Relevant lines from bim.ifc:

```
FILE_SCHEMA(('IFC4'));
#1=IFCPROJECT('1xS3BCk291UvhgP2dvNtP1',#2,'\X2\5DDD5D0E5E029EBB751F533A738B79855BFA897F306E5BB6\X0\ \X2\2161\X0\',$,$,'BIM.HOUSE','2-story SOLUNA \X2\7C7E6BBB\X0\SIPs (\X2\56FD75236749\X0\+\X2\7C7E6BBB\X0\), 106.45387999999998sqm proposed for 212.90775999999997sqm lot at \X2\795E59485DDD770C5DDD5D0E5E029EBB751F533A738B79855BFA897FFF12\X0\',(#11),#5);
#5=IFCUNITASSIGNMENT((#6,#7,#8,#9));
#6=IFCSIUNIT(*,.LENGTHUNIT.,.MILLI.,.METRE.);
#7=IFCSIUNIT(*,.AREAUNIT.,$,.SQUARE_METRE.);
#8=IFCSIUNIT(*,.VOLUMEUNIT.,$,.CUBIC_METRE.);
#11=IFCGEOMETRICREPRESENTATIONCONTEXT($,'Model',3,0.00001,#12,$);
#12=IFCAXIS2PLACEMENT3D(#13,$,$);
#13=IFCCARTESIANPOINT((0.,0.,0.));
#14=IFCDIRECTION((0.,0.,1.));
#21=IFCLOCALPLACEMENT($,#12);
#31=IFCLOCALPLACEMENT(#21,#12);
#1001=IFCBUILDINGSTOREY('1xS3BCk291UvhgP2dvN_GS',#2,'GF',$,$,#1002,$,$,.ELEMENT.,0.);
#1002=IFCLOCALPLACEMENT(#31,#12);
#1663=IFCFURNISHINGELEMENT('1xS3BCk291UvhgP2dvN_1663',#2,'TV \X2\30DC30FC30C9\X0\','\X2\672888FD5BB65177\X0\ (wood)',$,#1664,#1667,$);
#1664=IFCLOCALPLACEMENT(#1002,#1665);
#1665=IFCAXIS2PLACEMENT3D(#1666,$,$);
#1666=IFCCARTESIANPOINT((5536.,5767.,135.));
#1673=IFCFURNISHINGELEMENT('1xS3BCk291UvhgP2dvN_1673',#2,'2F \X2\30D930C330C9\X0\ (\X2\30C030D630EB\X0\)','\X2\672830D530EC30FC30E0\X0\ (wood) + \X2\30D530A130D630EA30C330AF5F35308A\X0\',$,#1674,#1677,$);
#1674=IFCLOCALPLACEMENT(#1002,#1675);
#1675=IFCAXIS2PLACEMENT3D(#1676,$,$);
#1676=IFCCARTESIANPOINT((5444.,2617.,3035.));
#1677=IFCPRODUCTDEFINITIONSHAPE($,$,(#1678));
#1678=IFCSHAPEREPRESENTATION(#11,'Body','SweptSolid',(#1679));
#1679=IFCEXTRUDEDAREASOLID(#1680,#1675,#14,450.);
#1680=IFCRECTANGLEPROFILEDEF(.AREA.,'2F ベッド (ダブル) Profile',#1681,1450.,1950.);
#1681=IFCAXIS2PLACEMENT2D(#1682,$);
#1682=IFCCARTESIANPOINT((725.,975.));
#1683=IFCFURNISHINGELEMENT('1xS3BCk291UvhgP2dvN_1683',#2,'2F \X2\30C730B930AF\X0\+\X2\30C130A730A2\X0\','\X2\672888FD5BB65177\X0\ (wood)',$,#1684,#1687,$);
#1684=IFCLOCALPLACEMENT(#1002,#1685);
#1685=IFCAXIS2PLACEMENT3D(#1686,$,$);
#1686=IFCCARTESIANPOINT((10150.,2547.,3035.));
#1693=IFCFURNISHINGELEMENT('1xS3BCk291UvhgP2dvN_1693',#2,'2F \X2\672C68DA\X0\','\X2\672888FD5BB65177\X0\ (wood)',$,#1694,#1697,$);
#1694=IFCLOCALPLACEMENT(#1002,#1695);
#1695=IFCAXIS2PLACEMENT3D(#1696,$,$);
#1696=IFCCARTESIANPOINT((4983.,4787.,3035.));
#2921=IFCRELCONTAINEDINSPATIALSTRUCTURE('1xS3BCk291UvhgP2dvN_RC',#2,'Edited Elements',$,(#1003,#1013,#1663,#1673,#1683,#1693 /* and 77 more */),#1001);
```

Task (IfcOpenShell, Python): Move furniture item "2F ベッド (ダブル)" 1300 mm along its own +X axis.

```python
import ifcopenshell
import ifcopenshell.api.geometry
import ifcopenshell.util.placement
import ifcopenshell.util.unit

model = ifcopenshell.open("bim.ifc")
unit_scale = ifcopenshell.util.unit.calculate_unit_scale(model)

item = model.by_id(1673)
matrix = ifcopenshell.util.placement.get_local_placement(item.ObjectPlacement)
matrix[:3, 3] += matrix[:3, 0] * 1.3 / unit_scale
ifcopenshell.api.geometry.edit_object_placement(model, product=item, matrix=matrix, is_si=False)

print(ifcopenshell.util.placement.get_local_placement(item.ObjectPlacement).round(3) + 0.0)

model.write("bim_rev.ifc")
```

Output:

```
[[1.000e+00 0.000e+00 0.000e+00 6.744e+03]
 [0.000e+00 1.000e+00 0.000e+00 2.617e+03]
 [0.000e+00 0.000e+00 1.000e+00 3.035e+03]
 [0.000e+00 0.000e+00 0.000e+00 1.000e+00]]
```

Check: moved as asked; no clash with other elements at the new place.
